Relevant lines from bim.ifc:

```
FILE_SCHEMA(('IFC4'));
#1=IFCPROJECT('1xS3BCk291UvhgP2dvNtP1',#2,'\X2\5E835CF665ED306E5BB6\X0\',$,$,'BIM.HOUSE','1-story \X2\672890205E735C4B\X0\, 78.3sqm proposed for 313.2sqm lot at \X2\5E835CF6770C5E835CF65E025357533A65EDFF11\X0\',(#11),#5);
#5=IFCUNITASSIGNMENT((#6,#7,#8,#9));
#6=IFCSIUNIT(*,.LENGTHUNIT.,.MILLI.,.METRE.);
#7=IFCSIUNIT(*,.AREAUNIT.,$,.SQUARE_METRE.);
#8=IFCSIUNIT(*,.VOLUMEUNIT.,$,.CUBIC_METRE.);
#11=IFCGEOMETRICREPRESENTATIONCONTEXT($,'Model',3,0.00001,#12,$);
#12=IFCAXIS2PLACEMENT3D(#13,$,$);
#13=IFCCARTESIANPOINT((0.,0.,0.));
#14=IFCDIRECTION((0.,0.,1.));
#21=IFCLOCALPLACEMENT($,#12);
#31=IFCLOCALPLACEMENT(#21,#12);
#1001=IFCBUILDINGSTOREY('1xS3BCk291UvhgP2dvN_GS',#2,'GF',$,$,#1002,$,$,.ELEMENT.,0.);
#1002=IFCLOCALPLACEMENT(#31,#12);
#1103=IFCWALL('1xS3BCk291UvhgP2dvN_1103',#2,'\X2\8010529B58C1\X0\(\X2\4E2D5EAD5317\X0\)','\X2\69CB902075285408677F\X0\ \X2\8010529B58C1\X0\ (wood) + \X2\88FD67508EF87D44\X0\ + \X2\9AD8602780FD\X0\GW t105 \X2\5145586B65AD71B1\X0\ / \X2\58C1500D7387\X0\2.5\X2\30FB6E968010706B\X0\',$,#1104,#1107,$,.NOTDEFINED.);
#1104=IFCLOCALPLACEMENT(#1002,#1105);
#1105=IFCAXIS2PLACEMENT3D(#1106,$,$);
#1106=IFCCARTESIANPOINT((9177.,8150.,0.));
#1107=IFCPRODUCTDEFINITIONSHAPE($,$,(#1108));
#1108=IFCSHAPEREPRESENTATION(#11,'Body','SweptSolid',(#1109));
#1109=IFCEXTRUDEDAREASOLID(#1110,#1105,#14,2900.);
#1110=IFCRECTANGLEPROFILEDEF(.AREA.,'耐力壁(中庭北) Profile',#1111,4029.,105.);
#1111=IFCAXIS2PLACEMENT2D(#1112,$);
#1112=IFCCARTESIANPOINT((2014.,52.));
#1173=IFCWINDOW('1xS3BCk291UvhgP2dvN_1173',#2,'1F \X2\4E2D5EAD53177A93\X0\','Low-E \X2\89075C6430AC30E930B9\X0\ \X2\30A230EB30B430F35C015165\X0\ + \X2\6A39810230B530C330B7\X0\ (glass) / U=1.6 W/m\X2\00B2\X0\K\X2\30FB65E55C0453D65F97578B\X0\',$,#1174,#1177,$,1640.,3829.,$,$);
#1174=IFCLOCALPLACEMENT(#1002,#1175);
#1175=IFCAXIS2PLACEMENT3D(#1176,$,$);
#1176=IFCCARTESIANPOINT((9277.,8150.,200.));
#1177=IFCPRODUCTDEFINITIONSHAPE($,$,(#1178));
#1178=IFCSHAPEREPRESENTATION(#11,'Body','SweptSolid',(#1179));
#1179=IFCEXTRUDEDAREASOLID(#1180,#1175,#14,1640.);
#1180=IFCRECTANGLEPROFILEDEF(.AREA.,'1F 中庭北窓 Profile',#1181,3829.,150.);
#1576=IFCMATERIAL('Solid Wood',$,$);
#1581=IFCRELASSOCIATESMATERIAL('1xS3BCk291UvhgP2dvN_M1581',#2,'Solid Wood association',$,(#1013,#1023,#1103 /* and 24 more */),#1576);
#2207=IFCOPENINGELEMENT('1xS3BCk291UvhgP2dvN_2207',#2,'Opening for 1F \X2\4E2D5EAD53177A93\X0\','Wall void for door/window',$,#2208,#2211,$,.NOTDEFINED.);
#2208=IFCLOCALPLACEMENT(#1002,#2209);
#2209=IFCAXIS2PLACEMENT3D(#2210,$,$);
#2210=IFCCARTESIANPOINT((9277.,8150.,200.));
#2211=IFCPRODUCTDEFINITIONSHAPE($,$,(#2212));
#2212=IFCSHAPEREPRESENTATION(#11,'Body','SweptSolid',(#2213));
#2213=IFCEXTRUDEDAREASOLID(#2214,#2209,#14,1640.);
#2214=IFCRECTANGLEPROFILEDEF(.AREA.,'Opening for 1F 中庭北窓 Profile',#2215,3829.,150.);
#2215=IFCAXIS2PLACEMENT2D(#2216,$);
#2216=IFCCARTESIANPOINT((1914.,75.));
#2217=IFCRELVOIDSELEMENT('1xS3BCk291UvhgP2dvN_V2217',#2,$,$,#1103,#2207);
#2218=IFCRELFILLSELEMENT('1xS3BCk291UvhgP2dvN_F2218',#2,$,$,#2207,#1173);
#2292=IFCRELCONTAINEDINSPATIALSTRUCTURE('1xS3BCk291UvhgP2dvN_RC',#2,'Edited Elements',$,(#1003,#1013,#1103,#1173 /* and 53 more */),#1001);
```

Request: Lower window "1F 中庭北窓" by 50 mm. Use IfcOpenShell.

```python
import numpy as np
import ifcopenshell
import ifcopenshell.api.geometry
import ifcopenshell.util.placement
import ifcopenshell.util.unit

model = ifcopenshell.open("bim.ifc")
unit_scale = ifcopenshell.util.unit.calculate_unit_scale(model)

window = model.by_guid("1xS3BCk291UvhgP2dvN_1173")
opening = window.FillsVoids[0].RelatingOpeningElement
dz = -0.05 / unit_scale

shift = np.array([0.0, 0.0, dz])
# The window is not placed relative to its opening, so move both.
for product in (opening, window):
    matrix = ifcopenshell.util.placement.get_local_placement(product.ObjectPlacement)
    matrix[:3, 3] += shift
    ifcopenshell.api.geometry.edit_object_placement(model, product=product, matrix=matrix, is_si=False)

print(f"moved by {dz * unit_scale:+.3f} m")

model.write("bim_updated.ifc")
```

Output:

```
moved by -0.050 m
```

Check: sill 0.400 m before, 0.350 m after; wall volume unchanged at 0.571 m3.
